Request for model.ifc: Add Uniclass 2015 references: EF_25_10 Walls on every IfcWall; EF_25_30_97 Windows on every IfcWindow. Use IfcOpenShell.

First a look at what the model holds.

```python
import ifcopenshell

model = ifcopenshell.open("model.ifc")
print(model.schema)
print("classifications:", [c.Name for c in model.by_type("IfcClassification")])
for ifc_class in ("IfcDoor", "IfcRoof", "IfcStair", "IfcWall", "IfcWindow"):
    print(ifc_class, len(model.by_type(ifc_class)))
```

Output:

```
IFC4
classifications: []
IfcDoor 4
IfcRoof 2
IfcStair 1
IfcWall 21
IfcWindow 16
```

```python
import ifcopenshell
import ifcopenshell.api.classification

model = ifcopenshell.open("model.ifc")

system = ifcopenshell.api.classification.add_classification(model, classification="Uniclass 2015")

codes = {
    "IfcWall": ("EF_25_10", "Walls"),
    "IfcWindow": ("EF_25_30_97", "Windows"),
}
for ifc_class, (code, name) in codes.items():
    products = model.by_type(ifc_class)
    ifcopenshell.api.classification.add_reference(
        model, products=products, classification=system, identification=code, name=name
    )
    print(code, len(products))

model.write("model-out.ifc")
```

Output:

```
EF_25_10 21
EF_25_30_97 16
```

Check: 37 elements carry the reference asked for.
